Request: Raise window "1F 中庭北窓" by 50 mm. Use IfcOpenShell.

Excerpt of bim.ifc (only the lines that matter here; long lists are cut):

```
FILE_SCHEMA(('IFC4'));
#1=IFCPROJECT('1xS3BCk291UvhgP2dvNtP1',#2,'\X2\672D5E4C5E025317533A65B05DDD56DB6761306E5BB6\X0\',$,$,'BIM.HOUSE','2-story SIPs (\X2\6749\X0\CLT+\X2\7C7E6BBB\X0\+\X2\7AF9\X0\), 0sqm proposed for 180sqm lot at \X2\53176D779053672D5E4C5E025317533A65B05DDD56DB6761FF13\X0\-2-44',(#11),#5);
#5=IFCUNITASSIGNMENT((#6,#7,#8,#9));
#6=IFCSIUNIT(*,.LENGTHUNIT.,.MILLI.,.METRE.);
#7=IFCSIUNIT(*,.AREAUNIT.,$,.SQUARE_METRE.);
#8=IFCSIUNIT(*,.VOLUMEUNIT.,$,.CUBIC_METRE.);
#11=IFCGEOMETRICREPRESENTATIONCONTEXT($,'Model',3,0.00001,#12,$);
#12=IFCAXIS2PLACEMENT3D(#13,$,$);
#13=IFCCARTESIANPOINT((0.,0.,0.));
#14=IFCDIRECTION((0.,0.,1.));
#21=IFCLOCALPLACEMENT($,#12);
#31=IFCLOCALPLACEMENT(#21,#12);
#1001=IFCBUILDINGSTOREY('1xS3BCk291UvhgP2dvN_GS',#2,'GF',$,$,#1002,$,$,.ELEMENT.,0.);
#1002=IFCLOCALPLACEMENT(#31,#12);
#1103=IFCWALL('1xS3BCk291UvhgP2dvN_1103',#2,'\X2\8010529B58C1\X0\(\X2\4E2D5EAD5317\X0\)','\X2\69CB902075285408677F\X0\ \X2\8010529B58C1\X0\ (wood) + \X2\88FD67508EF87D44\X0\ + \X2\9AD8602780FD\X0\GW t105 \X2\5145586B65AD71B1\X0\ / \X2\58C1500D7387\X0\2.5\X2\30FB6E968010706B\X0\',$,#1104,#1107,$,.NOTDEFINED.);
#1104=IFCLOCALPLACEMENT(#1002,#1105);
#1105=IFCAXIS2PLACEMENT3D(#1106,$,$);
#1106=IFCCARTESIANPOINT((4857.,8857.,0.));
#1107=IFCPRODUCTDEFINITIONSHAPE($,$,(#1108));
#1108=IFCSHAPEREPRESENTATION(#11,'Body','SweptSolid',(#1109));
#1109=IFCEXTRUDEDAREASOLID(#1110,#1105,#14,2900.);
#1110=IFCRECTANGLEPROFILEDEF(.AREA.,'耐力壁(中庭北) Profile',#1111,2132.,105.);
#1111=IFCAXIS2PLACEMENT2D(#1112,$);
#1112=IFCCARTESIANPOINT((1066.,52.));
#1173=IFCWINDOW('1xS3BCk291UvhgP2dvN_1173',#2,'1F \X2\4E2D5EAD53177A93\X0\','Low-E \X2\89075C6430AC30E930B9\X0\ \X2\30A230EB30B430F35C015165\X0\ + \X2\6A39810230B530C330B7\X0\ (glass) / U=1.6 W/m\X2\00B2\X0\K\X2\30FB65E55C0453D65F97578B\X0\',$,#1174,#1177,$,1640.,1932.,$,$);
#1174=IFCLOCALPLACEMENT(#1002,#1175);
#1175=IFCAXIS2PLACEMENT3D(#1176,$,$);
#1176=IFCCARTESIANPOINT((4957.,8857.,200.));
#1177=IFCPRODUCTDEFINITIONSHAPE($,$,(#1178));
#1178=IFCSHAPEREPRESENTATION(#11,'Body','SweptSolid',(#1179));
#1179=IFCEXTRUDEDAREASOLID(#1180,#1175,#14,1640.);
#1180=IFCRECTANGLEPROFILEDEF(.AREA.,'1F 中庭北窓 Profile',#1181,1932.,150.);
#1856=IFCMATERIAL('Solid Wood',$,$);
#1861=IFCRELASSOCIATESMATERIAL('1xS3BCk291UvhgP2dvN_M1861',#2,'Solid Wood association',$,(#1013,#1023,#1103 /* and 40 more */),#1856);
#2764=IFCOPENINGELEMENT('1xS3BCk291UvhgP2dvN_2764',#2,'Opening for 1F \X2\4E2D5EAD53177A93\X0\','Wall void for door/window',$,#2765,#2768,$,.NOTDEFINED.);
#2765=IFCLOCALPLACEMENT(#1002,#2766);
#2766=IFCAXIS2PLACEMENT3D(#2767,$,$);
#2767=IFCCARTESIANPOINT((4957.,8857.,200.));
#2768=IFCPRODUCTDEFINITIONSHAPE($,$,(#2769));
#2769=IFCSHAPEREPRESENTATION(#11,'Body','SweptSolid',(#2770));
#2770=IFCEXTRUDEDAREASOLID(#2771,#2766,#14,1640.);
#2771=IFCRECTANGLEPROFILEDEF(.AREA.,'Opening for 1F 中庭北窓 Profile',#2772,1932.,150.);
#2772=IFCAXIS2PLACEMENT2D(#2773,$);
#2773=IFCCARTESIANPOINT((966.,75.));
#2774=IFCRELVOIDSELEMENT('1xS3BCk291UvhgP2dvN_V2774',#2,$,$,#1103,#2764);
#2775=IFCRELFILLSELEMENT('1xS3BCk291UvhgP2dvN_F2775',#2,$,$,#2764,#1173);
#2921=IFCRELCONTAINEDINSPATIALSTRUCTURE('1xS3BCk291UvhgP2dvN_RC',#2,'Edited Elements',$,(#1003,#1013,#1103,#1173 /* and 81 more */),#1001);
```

```python
import numpy as np
import ifcopenshell
import ifcopenshell.api.geometry
import ifcopenshell.util.placement
import ifcopenshell.util.unit

model = ifcopenshell.open("bim.ifc")
unit_scale = ifcopenshell.util.unit.calculate_unit_scale(model)

window = model.by_guid("1xS3BCk291UvhgP2dvN_1173")
opening = window.FillsVoids[0].RelatingOpeningElement
dz = 50.0

shift = np.array([0.0, 0.0, dz])
# The window is not placed relative to its opening, so move both.
for product in (opening, window):
    matrix = ifcopenshell.util.placement.get_local_placement(product.ObjectPlacement)
    matrix[:3, 3] += shift
    ifcopenshell.api.geometry.edit_object_placement(model, product=product, matrix=matrix, is_si=False)

print(f"moved by {dz * unit_scale:+.3f} m")

model.write("bim-out.ifc")
```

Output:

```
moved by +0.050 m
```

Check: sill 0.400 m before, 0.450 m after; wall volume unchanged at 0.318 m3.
